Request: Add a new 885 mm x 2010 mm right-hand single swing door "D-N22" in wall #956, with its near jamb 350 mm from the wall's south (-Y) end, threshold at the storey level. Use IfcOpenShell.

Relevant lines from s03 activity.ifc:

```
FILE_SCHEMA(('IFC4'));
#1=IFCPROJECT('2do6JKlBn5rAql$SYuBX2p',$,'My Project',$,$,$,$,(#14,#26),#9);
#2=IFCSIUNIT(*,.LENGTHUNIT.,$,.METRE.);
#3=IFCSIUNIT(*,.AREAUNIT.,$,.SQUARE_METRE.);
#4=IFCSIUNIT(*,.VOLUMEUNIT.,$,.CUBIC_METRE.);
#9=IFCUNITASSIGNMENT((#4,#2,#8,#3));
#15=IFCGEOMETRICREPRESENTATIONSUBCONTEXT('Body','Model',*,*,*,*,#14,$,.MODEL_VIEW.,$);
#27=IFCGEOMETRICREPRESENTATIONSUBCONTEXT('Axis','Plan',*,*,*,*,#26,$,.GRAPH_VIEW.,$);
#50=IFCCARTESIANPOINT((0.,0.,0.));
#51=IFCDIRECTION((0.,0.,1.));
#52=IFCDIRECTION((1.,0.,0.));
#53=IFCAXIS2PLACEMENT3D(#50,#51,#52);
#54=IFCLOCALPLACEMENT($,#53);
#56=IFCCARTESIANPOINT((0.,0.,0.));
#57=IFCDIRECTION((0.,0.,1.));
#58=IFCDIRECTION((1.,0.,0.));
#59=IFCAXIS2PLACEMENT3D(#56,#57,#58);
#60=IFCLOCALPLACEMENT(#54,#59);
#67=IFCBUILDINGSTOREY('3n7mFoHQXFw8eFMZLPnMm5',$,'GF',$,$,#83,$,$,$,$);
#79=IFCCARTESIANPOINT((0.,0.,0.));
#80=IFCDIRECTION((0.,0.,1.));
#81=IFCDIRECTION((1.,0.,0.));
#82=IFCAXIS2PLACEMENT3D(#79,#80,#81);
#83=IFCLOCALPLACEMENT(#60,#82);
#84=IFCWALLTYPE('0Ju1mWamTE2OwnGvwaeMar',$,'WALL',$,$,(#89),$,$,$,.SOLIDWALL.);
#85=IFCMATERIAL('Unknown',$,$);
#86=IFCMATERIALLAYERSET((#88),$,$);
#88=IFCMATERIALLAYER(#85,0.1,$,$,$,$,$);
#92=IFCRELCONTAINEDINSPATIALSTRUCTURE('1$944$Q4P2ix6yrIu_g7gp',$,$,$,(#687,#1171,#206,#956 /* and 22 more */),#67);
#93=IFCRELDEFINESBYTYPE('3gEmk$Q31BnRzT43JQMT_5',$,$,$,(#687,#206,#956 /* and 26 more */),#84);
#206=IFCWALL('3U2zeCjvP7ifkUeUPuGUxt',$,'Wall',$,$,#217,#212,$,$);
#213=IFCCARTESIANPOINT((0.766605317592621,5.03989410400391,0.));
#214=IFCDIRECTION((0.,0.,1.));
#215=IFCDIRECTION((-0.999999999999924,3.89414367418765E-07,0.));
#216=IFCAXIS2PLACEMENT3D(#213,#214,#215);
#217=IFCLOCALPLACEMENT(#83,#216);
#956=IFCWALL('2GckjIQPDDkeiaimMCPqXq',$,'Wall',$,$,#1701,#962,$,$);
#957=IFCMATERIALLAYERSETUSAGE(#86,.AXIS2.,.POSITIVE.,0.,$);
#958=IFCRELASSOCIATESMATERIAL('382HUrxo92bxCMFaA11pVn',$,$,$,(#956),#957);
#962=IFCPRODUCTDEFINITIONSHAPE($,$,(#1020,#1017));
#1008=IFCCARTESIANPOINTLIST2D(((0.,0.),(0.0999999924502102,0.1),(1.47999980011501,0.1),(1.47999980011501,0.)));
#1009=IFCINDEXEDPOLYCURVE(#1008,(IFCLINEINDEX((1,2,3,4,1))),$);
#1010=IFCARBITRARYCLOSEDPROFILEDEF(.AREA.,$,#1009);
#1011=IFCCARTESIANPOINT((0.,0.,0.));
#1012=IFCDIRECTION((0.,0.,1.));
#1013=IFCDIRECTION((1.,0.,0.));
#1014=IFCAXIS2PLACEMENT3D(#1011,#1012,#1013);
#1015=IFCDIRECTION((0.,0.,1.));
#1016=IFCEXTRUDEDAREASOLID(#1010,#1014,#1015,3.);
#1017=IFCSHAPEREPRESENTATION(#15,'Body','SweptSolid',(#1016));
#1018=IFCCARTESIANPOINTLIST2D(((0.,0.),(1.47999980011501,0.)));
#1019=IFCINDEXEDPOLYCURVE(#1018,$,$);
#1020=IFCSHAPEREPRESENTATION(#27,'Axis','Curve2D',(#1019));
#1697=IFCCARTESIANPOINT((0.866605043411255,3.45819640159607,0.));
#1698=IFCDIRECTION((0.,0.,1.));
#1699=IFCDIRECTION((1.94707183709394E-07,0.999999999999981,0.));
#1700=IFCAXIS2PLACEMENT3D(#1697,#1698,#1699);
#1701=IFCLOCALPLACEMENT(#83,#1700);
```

```python
import numpy as np
import ifcopenshell
import ifcopenshell.api.feature
import ifcopenshell.api.geometry
import ifcopenshell.api.root
import ifcopenshell.api.spatial
import ifcopenshell.geom
import ifcopenshell.util.element
import ifcopenshell.util.placement
import ifcopenshell.util.representation
import ifcopenshell.util.shape
import ifcopenshell.util.unit

model = ifcopenshell.open("s03 activity.ifc")
unit_scale = ifcopenshell.util.unit.calculate_unit_scale(model)
settings = ifcopenshell.geom.settings()


def volume(element):
    """Net volume in cubic metres, openings subtracted."""
    shape = ifcopenshell.geom.create_shape(settings, element)
    return ifcopenshell.util.shape.get_volume(shape.geometry)


wall = model.by_id(956)
storey = ifcopenshell.util.element.get_container(wall, ifc_class="IfcBuildingStorey")
context = ifcopenshell.util.representation.get_context(model, "Model", "Body", "MODEL_VIEW")
before = volume(wall)

width, height, from_end, sill = 0.885, 2.01, 0.35, 0.0  # metres

# The wall runs along its own X axis, and the end named is its -X end.
wall_shape = ifcopenshell.geom.create_shape(settings, wall)
x, y, z = ifcopenshell.util.shape.get_vertices(wall_shape.geometry).T
start = x.min() + from_end
face, thickness = float(y.min()), float(y.max() - y.min())
wall_matrix = ifcopenshell.util.placement.get_local_placement(wall.ObjectPlacement)
level = ifcopenshell.util.placement.get_local_placement(storey.ObjectPlacement)[2, 3]


def in_wall(x, y):
    """Placement at x, y metres in the wall's axes, at sill height."""
    matrix = wall_matrix.copy()
    matrix[:, 3] = wall_matrix @ np.array([x / unit_scale, y / unit_scale, 0.0, 1.0])
    matrix[2, 3] = level + sill / unit_scale
    return matrix


# Opening: a box that overshoots both wall faces by 50 mm.
opening = ifcopenshell.api.root.create_entity(model, ifc_class="IfcOpeningElement", predefined_type="OPENING")
box = ifcopenshell.api.geometry.add_wall_representation(
    model, context=context, length=width, height=height, thickness=thickness + 0.1
)
ifcopenshell.api.geometry.assign_representation(model, product=opening, representation=box)
ifcopenshell.api.geometry.edit_object_placement(model, product=opening, matrix=in_wall(start, face - 0.05), is_si=False)
ifcopenshell.api.feature.add_feature(model, feature=opening, element=wall)

door = ifcopenshell.api.root.create_entity(model, ifc_class="IfcDoor", name="D-N22", predefined_type="DOOR")
door.OverallWidth, door.OverallHeight = width / unit_scale, height / unit_scale
door.OperationType = "SINGLE_SWING_RIGHT"
body = ifcopenshell.api.geometry.add_door_representation(
    model,
    context=context,
    overall_width=door.OverallWidth,
    overall_height=door.OverallHeight,
    operation_type="SINGLE_SWING_RIGHT",
    lining_properties={"LiningDepth": thickness / unit_scale, "ThresholdDepth": thickness / unit_scale},
)
ifcopenshell.api.geometry.assign_representation(model, product=door, representation=body)
ifcopenshell.api.spatial.assign_container(model, products=[door], relating_structure=storey)
ifcopenshell.api.feature.add_filling(model, opening=opening, element=door)

# The lining spans the wall, so the door starts at the wall face.
ifcopenshell.api.geometry.edit_object_placement(model, product=door, matrix=in_wall(start, face), is_si=False)

after = volume(wall)

print(f"wall volume {before:.3f} -> {after:.3f} m3")

model.write("s03 activity_edited.ifc")
```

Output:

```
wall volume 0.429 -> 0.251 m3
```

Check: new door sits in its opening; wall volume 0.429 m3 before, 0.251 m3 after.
